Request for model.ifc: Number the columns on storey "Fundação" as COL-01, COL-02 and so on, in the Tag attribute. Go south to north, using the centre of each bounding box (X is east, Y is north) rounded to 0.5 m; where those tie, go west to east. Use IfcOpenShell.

First a look at what the model holds.

```python
import ifcopenshell
import ifcopenshell.util.element
import ifcopenshell.util.placement

model = ifcopenshell.open("model.ifc")
print(model.schema)
storey = next(s for s in model.by_type("IfcBuildingStorey") if s.Name == "Fundação")
columns = [e for e in ifcopenshell.util.element.get_decomposition(storey) if e.is_a("IfcColumn")]
for e in sorted(columns, key=lambda e: e.id()):
    origin = ifcopenshell.util.placement.get_local_placement(e.ObjectPlacement)[:3, 3]
    print(e.id(), e.Tag, e.Name, origin.round(2) + 0.0, sep=" | ")
```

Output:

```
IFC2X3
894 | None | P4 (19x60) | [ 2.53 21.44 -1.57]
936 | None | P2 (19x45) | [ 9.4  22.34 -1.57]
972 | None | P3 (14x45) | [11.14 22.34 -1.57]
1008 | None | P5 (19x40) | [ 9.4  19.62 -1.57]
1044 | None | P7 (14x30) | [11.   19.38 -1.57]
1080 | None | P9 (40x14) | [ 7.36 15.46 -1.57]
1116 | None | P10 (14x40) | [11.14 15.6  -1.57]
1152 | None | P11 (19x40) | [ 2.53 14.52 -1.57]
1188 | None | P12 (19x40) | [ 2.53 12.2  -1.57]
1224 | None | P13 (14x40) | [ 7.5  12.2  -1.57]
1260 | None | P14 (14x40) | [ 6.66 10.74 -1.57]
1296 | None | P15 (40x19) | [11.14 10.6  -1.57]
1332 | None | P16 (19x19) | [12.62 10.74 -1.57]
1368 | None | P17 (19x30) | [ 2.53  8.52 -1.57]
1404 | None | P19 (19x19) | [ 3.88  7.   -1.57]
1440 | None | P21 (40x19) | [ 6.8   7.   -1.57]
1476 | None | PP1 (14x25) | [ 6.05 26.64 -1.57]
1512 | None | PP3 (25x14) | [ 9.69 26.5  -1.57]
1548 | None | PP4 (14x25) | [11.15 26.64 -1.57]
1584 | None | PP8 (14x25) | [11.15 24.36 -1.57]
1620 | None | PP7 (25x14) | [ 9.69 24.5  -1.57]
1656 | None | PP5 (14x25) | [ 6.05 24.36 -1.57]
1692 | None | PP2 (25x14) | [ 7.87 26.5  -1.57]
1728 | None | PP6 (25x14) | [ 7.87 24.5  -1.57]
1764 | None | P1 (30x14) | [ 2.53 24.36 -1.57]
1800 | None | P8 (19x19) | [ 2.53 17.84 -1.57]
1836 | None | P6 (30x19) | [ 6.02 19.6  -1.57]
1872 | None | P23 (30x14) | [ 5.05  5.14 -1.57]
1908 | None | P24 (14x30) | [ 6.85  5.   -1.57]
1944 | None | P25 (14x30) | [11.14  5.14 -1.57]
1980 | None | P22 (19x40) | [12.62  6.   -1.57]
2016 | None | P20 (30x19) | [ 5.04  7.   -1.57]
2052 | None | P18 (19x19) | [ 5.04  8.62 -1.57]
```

```python
import ifcopenshell
import ifcopenshell.geom
import ifcopenshell.util.element
import ifcopenshell.util.shape

model = ifcopenshell.open("model.ifc")
settings = ifcopenshell.geom.settings()
settings.set("use-world-coords", True)


def centre(element):
    shape = ifcopenshell.geom.create_shape(settings, element)
    return ifcopenshell.util.shape.get_bbox_centroid(shape.geometry)


storey = next(s for s in model.by_type("IfcBuildingStorey") if s.Name == "Fundação")
columns = [e for e in ifcopenshell.util.element.get_decomposition(storey) if e.is_a("IfcColumn")]

# Insertion points can sit at a corner or the storey origin, so sort by the geometry (in metres).
centres = {e: centre(e) for e in columns}
columns.sort(key=lambda e: (round(centres[e][1] / 0.5), centres[e][0]))

for i, e in enumerate(columns, start=1):
    number = f"COL-{i:02d}"
    e.Tag = number
    print(e.id(), number)

model.write("model_v2.ifc")
```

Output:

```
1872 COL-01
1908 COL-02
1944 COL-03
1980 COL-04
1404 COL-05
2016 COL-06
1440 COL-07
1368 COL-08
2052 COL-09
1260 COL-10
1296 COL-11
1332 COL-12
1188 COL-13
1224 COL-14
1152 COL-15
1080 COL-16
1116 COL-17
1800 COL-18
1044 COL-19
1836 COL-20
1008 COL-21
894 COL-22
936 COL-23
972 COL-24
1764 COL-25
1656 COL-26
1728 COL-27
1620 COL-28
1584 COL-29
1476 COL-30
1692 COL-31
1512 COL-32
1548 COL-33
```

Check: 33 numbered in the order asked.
